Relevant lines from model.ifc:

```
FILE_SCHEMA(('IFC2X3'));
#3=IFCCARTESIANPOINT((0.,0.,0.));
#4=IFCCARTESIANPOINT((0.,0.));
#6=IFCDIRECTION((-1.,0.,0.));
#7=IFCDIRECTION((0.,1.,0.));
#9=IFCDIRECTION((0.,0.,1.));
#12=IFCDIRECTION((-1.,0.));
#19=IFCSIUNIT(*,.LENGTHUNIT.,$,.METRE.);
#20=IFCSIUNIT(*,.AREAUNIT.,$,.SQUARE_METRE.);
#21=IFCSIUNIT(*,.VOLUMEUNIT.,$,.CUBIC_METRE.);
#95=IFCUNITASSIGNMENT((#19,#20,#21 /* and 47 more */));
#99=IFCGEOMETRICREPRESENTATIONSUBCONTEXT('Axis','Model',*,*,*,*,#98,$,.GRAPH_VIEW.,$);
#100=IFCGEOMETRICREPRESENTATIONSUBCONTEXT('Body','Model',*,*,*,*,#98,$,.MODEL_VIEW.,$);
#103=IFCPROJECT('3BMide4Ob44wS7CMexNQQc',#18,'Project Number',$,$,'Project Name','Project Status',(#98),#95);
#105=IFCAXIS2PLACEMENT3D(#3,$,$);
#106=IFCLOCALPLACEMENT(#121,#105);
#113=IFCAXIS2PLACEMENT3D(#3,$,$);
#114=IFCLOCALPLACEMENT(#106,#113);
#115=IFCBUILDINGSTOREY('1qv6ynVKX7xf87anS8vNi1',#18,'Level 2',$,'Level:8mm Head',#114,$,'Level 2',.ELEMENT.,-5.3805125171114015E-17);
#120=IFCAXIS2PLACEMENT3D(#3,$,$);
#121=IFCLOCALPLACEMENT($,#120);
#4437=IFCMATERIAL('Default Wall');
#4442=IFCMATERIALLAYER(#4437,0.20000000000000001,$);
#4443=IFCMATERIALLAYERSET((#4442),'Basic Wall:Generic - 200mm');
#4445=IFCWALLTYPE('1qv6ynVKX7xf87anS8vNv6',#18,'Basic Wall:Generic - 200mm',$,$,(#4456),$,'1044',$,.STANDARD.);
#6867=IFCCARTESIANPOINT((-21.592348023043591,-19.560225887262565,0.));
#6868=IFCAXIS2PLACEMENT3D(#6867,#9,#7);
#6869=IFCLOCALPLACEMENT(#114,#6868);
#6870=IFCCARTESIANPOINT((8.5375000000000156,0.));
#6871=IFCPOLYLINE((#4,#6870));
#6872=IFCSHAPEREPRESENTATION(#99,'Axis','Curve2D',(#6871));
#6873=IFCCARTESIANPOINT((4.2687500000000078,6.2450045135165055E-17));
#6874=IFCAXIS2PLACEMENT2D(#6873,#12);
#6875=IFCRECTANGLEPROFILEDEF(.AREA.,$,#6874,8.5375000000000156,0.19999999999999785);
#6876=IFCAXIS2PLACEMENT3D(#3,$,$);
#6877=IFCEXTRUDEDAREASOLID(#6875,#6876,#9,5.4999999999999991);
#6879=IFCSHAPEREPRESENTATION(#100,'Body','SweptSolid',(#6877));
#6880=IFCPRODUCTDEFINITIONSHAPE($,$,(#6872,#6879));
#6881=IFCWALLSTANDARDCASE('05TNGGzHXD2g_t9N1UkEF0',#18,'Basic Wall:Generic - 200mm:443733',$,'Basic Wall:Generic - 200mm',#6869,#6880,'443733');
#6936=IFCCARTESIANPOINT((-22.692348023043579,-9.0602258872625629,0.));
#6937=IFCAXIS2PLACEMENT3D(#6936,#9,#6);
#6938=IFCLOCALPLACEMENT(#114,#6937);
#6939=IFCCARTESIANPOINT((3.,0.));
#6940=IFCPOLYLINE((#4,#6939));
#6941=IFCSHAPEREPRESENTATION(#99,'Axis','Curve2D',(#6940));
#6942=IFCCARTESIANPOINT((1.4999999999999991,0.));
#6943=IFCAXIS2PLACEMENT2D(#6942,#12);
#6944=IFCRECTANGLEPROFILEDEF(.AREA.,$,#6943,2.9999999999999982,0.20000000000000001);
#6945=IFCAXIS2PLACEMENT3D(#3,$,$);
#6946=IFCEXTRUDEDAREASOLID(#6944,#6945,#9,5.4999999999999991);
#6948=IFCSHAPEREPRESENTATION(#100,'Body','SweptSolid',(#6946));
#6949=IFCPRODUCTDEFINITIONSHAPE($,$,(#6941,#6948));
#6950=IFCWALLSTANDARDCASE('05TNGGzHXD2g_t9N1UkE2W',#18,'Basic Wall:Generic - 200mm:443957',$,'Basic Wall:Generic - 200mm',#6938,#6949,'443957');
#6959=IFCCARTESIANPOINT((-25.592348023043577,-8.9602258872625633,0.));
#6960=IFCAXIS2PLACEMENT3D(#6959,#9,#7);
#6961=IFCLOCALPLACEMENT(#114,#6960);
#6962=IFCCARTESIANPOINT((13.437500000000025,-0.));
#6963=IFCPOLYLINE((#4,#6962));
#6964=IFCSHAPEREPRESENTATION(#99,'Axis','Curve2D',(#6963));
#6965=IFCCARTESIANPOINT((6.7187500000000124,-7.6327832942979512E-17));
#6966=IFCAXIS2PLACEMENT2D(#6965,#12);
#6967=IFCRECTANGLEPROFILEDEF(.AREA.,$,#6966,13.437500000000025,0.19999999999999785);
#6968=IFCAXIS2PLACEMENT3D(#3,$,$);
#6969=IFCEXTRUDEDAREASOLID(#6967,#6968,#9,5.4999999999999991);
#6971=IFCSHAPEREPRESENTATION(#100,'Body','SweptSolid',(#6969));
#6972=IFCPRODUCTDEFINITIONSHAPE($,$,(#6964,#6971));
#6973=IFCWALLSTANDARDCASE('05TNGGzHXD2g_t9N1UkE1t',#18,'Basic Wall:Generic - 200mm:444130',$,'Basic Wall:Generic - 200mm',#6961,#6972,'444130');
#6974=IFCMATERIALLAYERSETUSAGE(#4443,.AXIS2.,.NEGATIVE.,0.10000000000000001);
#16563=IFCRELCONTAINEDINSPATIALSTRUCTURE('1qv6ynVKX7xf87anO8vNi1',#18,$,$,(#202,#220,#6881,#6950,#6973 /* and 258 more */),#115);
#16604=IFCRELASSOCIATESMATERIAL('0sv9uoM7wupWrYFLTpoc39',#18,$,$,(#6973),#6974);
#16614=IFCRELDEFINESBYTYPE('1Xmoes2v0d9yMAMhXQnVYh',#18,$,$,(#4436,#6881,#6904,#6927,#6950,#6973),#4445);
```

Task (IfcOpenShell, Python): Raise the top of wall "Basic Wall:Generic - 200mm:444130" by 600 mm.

```python
import ifcopenshell
import ifcopenshell.geom
import ifcopenshell.util.representation
import ifcopenshell.util.shape

model = ifcopenshell.open("model.ifc")
settings = ifcopenshell.geom.settings()


def volume(element):
    """Net volume in cubic metres, openings subtracted."""
    shape = ifcopenshell.geom.create_shape(settings, element)
    return ifcopenshell.util.shape.get_volume(shape.geometry)


wall = model.by_id(6973)
before = volume(wall)

body = ifcopenshell.util.representation.get_representation(wall, "Model", "Body")
solid = body.Items[0]
old_height = solid.Depth
solid.Depth += 0.6
after = volume(wall)

print(f"height {old_height:g} -> {solid.Depth:g}, volume {before:.3f} -> {after:.3f} m3")

model.write("model_edited.ifc")
```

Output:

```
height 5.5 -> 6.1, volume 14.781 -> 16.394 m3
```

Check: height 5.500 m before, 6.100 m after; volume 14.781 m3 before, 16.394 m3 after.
